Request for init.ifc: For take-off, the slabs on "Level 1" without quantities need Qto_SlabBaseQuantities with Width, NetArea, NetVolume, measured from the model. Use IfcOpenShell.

First a look at what the model holds.

```python
import ifcopenshell
import ifcopenshell.util.element
import ifcopenshell.util.unit

model = ifcopenshell.open("init.ifc")
print(model.schema)
for unit_type in ("LENGTHUNIT", "AREAUNIT", "VOLUMEUNIT"):
    print(unit_type, ifcopenshell.util.unit.calculate_unit_scale(model, unit_type))
storey = next(s for s in model.by_type("IfcBuildingStorey") if s.Name == "Level 1")
slabs = [e for e in ifcopenshell.util.element.get_decomposition(storey) if e.is_a("IfcSlab")]
for e in sorted(slabs, key=lambda e: e.id()):
    print(e.id(), e.is_a(), e.Name, list(ifcopenshell.util.element.get_psets(e, qtos_only=True)), sep=" | ")
```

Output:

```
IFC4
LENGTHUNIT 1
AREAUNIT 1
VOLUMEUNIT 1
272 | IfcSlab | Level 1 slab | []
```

```python
import ifcopenshell
import ifcopenshell.api.pset
import ifcopenshell.geom
import ifcopenshell.util.element
import ifcopenshell.util.shape
import ifcopenshell.util.unit

model = ifcopenshell.open("init.ifc")
unit_scale = ifcopenshell.util.unit.calculate_unit_scale(model)
area_scale = ifcopenshell.util.unit.calculate_unit_scale(model, "AREAUNIT")
volume_scale = ifcopenshell.util.unit.calculate_unit_scale(model, "VOLUMEUNIT")
settings = ifcopenshell.geom.settings()

storey = next(s for s in model.by_type("IfcBuildingStorey") if s.Name == "Level 1")
slabs = [e for e in ifcopenshell.util.element.get_decomposition(storey) if e.is_a("IfcSlab")]

for e in sorted(slabs, key=lambda e: e.id()):
    if ifcopenshell.util.element.get_psets(e, qtos_only=True, should_inherit=False):
        continue
    # Geometry comes back in metres, in the element's own axes.
    shape = ifcopenshell.geom.create_shape(settings, e)
    values = {
        "Width": ifcopenshell.util.shape.get_z(shape.geometry) / unit_scale,
        "NetArea": ifcopenshell.util.shape.get_footprint_area(shape.geometry) / area_scale,
        "NetVolume": ifcopenshell.util.shape.get_volume(shape.geometry) / volume_scale,
    }
    qto = ifcopenshell.api.pset.add_qto(model, product=e, name="Qto_SlabBaseQuantities")
    ifcopenshell.api.pset.edit_qto(model, qto=qto, properties=values)
    print(e.id(), {k: round(v, 3) for k, v in values.items()})

model.write("init_updated.ifc")
```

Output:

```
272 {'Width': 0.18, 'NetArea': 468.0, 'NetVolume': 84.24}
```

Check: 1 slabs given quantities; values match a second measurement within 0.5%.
